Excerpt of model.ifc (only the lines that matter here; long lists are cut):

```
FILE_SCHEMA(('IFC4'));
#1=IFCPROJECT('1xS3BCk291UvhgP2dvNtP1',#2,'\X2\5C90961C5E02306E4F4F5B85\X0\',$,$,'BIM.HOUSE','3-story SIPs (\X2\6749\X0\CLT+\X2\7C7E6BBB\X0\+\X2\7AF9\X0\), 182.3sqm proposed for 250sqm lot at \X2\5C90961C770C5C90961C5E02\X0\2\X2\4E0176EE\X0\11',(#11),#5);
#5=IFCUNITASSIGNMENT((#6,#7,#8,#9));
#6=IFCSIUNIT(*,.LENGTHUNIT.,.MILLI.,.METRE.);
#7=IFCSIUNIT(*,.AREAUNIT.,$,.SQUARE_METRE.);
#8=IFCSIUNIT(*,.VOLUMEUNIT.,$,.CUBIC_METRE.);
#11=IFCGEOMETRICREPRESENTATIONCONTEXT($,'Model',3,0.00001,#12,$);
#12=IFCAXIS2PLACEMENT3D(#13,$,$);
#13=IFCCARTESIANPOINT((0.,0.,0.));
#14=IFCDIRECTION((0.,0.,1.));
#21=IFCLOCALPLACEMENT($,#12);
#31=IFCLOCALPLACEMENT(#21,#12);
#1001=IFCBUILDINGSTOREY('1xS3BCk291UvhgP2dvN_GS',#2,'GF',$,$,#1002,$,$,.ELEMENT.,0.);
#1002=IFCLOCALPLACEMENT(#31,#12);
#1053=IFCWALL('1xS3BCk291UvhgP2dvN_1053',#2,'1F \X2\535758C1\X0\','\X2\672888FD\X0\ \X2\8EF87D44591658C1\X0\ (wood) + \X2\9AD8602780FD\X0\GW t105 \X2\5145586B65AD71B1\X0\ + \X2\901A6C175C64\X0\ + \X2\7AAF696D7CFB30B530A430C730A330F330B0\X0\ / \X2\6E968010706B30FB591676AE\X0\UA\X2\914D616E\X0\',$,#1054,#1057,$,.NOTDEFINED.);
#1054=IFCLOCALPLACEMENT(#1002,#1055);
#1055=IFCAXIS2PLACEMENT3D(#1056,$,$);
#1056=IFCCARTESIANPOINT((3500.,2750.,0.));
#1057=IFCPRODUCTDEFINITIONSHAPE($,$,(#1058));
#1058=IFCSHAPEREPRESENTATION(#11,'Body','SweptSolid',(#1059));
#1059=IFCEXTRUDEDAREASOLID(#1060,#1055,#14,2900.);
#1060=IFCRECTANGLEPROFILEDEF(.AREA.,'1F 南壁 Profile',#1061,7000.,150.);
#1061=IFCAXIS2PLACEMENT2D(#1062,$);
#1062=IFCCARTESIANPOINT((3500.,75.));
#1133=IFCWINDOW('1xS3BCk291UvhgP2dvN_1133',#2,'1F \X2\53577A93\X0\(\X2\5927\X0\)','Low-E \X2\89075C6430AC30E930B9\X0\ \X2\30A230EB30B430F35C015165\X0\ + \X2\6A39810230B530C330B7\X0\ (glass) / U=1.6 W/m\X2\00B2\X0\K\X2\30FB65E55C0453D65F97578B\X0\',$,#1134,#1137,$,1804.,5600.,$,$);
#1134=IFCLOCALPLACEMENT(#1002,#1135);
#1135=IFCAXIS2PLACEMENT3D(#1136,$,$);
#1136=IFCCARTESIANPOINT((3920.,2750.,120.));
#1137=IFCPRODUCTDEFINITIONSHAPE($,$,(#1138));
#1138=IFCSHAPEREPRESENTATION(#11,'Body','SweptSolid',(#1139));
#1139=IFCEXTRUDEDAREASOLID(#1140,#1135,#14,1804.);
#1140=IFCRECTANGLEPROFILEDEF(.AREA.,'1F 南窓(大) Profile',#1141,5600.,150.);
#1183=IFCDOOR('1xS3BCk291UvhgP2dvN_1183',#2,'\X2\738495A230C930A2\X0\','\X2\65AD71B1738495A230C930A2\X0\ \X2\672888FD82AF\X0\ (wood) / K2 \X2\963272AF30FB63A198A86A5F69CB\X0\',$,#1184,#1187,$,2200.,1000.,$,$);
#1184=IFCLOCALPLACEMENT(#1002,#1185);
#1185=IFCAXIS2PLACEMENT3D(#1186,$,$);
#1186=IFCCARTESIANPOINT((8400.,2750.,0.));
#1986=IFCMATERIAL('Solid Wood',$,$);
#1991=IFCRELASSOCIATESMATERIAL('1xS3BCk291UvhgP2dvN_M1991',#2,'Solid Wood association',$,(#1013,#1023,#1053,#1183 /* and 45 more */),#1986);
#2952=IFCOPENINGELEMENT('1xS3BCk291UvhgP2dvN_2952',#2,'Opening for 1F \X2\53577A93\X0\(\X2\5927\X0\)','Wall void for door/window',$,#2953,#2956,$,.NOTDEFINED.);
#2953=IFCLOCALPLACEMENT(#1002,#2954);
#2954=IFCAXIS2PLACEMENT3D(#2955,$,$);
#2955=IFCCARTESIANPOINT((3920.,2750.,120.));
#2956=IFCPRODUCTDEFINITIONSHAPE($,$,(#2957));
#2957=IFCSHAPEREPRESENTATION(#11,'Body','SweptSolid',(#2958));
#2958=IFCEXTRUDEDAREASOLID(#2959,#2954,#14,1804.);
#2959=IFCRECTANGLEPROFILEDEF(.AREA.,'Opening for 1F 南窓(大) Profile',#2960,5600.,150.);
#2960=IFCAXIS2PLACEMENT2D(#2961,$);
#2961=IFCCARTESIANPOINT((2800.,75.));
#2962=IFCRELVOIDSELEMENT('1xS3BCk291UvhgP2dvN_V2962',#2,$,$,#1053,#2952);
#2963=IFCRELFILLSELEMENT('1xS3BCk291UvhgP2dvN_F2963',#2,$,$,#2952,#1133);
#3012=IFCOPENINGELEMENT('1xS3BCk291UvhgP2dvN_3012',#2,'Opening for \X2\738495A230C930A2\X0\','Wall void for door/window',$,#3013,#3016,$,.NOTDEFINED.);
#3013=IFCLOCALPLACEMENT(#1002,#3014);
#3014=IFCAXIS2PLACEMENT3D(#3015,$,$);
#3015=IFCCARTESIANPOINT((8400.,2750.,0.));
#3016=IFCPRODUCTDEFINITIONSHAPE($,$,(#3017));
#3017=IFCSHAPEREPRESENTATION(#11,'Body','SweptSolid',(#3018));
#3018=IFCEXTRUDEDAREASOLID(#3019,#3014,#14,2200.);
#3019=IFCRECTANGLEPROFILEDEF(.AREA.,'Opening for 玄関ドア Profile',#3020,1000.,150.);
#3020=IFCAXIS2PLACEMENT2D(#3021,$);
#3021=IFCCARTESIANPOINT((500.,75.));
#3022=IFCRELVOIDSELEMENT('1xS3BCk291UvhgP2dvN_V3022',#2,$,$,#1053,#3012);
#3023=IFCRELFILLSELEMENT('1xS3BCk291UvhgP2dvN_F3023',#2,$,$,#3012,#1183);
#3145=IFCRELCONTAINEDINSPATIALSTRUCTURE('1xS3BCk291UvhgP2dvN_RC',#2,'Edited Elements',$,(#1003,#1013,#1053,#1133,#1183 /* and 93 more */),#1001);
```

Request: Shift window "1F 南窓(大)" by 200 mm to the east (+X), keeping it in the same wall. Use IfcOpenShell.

```python
import ifcopenshell
import ifcopenshell.api.geometry
import ifcopenshell.util.placement
import ifcopenshell.util.unit

model = ifcopenshell.open("model.ifc")
unit_scale = ifcopenshell.util.unit.calculate_unit_scale(model)

window = model.by_guid("1xS3BCk291UvhgP2dvN_1133")
opening = window.FillsVoids[0].RelatingOpeningElement
wall = opening.VoidsElements[0].RelatingBuildingElement

wall_matrix = ifcopenshell.util.placement.get_local_placement(wall.ObjectPlacement)
shift = wall_matrix[:3, 0] * 0.2 / unit_scale
before = ifcopenshell.util.placement.get_local_placement(window.ObjectPlacement)[:3, 3].copy()

# The window is not placed relative to its opening, so move both.
for product in (opening, window):
    matrix = ifcopenshell.util.placement.get_local_placement(product.ObjectPlacement)
    matrix[:3, 3] += shift
    ifcopenshell.api.geometry.edit_object_placement(model, product=product, matrix=matrix, is_si=False)

after = ifcopenshell.util.placement.get_local_placement(window.ObjectPlacement)[:3, 3]
print("window moved by", (after - before).round(3) + 0.0)

model.write("model_updated.ifc")
```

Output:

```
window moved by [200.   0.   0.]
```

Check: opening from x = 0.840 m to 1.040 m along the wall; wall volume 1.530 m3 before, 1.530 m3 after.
